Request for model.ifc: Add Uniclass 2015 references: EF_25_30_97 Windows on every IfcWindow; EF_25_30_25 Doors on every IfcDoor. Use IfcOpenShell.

First a look at what the model holds.

```python
import ifcopenshell

model = ifcopenshell.open("model.ifc")
print(model.schema)
print("classifications:", [c.Name for c in model.by_type("IfcClassification")])
for ifc_class in ("IfcDoor", "IfcRoof", "IfcStair", "IfcWall", "IfcWindow"):
    print(ifc_class, len(model.by_type(ifc_class)))
```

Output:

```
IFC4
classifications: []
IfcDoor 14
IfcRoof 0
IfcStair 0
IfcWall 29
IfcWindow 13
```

```python
import ifcopenshell
import ifcopenshell.api.classification

model = ifcopenshell.open("model.ifc")

system = ifcopenshell.api.classification.add_classification(model, classification="Uniclass 2015")

codes = {
    "IfcWindow": ("EF_25_30_97", "Windows"),
    "IfcDoor": ("EF_25_30_25", "Doors"),
}
for ifc_class, (code, name) in codes.items():
    products = model.by_type(ifc_class)
    ifcopenshell.api.classification.add_reference(
        model, products=products, classification=system, identification=code, name=name
    )
    print(code, len(products))

model.write("model_rev.ifc")
```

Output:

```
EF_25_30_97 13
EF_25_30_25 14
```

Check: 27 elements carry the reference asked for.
